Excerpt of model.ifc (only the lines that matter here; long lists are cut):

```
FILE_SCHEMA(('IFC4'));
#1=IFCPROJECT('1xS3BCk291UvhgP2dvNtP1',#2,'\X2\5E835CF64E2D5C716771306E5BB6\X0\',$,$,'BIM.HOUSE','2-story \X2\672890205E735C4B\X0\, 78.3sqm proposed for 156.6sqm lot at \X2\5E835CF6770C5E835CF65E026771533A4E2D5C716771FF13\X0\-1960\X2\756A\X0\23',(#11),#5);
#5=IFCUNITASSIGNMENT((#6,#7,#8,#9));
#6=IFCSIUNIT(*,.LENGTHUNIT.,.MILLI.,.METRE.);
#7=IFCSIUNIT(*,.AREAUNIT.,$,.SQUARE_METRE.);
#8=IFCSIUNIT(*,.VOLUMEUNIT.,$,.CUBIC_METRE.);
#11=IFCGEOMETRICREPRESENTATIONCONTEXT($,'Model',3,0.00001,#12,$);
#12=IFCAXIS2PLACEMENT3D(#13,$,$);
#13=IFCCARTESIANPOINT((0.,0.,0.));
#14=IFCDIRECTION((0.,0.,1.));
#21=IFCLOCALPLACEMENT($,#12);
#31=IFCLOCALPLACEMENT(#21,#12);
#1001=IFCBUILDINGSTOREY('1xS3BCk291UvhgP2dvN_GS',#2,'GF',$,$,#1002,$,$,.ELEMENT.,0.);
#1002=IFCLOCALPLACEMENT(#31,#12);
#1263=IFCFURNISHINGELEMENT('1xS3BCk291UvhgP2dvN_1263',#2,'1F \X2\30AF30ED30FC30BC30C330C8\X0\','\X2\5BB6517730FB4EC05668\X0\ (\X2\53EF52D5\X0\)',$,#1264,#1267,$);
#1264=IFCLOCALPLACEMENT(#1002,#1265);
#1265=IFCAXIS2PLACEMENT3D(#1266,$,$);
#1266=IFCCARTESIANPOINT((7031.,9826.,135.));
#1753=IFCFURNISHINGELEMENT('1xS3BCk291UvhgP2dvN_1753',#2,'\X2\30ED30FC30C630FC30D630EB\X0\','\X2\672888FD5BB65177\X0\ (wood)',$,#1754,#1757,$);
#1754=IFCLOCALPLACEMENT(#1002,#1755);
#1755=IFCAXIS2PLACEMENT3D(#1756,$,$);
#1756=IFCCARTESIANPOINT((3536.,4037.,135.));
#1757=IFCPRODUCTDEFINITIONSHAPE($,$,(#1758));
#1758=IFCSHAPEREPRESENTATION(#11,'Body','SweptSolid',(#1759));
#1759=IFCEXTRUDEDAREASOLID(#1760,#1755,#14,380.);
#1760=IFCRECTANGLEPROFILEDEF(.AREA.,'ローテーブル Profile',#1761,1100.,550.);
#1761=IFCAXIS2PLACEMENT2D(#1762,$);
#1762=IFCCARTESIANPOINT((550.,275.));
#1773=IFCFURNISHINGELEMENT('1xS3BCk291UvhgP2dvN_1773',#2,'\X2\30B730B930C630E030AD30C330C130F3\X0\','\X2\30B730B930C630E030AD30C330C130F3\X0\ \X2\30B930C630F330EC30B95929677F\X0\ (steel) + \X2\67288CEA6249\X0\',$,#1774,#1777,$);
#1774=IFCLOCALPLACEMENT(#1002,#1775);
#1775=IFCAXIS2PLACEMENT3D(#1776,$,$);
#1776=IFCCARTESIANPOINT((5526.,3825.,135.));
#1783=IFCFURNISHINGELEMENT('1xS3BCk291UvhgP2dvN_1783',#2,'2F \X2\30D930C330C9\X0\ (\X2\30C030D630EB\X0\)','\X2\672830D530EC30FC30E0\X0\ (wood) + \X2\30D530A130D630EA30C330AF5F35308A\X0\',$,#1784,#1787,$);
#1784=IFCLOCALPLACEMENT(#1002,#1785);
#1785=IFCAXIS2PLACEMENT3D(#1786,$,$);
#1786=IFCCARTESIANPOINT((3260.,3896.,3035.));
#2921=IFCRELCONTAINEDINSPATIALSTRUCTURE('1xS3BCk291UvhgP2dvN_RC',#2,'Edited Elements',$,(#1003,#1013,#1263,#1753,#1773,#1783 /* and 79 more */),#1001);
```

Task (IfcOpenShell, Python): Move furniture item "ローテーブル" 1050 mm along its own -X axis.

```python
import ifcopenshell
import ifcopenshell.api.geometry
import ifcopenshell.util.placement

model = ifcopenshell.open("model.ifc")

item = model.by_id(1753)
matrix = ifcopenshell.util.placement.get_local_placement(item.ObjectPlacement)
matrix[:3, 3] -= matrix[:3, 0] * 1050.0
ifcopenshell.api.geometry.edit_object_placement(model, product=item, matrix=matrix, is_si=False)

print(ifcopenshell.util.placement.get_local_placement(item.ObjectPlacement).round(3) + 0.0)

model.write("model-out.ifc")
```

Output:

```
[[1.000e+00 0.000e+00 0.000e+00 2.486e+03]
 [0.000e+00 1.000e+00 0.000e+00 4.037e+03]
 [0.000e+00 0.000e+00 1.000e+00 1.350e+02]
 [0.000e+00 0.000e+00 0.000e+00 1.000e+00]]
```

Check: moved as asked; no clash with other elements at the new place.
